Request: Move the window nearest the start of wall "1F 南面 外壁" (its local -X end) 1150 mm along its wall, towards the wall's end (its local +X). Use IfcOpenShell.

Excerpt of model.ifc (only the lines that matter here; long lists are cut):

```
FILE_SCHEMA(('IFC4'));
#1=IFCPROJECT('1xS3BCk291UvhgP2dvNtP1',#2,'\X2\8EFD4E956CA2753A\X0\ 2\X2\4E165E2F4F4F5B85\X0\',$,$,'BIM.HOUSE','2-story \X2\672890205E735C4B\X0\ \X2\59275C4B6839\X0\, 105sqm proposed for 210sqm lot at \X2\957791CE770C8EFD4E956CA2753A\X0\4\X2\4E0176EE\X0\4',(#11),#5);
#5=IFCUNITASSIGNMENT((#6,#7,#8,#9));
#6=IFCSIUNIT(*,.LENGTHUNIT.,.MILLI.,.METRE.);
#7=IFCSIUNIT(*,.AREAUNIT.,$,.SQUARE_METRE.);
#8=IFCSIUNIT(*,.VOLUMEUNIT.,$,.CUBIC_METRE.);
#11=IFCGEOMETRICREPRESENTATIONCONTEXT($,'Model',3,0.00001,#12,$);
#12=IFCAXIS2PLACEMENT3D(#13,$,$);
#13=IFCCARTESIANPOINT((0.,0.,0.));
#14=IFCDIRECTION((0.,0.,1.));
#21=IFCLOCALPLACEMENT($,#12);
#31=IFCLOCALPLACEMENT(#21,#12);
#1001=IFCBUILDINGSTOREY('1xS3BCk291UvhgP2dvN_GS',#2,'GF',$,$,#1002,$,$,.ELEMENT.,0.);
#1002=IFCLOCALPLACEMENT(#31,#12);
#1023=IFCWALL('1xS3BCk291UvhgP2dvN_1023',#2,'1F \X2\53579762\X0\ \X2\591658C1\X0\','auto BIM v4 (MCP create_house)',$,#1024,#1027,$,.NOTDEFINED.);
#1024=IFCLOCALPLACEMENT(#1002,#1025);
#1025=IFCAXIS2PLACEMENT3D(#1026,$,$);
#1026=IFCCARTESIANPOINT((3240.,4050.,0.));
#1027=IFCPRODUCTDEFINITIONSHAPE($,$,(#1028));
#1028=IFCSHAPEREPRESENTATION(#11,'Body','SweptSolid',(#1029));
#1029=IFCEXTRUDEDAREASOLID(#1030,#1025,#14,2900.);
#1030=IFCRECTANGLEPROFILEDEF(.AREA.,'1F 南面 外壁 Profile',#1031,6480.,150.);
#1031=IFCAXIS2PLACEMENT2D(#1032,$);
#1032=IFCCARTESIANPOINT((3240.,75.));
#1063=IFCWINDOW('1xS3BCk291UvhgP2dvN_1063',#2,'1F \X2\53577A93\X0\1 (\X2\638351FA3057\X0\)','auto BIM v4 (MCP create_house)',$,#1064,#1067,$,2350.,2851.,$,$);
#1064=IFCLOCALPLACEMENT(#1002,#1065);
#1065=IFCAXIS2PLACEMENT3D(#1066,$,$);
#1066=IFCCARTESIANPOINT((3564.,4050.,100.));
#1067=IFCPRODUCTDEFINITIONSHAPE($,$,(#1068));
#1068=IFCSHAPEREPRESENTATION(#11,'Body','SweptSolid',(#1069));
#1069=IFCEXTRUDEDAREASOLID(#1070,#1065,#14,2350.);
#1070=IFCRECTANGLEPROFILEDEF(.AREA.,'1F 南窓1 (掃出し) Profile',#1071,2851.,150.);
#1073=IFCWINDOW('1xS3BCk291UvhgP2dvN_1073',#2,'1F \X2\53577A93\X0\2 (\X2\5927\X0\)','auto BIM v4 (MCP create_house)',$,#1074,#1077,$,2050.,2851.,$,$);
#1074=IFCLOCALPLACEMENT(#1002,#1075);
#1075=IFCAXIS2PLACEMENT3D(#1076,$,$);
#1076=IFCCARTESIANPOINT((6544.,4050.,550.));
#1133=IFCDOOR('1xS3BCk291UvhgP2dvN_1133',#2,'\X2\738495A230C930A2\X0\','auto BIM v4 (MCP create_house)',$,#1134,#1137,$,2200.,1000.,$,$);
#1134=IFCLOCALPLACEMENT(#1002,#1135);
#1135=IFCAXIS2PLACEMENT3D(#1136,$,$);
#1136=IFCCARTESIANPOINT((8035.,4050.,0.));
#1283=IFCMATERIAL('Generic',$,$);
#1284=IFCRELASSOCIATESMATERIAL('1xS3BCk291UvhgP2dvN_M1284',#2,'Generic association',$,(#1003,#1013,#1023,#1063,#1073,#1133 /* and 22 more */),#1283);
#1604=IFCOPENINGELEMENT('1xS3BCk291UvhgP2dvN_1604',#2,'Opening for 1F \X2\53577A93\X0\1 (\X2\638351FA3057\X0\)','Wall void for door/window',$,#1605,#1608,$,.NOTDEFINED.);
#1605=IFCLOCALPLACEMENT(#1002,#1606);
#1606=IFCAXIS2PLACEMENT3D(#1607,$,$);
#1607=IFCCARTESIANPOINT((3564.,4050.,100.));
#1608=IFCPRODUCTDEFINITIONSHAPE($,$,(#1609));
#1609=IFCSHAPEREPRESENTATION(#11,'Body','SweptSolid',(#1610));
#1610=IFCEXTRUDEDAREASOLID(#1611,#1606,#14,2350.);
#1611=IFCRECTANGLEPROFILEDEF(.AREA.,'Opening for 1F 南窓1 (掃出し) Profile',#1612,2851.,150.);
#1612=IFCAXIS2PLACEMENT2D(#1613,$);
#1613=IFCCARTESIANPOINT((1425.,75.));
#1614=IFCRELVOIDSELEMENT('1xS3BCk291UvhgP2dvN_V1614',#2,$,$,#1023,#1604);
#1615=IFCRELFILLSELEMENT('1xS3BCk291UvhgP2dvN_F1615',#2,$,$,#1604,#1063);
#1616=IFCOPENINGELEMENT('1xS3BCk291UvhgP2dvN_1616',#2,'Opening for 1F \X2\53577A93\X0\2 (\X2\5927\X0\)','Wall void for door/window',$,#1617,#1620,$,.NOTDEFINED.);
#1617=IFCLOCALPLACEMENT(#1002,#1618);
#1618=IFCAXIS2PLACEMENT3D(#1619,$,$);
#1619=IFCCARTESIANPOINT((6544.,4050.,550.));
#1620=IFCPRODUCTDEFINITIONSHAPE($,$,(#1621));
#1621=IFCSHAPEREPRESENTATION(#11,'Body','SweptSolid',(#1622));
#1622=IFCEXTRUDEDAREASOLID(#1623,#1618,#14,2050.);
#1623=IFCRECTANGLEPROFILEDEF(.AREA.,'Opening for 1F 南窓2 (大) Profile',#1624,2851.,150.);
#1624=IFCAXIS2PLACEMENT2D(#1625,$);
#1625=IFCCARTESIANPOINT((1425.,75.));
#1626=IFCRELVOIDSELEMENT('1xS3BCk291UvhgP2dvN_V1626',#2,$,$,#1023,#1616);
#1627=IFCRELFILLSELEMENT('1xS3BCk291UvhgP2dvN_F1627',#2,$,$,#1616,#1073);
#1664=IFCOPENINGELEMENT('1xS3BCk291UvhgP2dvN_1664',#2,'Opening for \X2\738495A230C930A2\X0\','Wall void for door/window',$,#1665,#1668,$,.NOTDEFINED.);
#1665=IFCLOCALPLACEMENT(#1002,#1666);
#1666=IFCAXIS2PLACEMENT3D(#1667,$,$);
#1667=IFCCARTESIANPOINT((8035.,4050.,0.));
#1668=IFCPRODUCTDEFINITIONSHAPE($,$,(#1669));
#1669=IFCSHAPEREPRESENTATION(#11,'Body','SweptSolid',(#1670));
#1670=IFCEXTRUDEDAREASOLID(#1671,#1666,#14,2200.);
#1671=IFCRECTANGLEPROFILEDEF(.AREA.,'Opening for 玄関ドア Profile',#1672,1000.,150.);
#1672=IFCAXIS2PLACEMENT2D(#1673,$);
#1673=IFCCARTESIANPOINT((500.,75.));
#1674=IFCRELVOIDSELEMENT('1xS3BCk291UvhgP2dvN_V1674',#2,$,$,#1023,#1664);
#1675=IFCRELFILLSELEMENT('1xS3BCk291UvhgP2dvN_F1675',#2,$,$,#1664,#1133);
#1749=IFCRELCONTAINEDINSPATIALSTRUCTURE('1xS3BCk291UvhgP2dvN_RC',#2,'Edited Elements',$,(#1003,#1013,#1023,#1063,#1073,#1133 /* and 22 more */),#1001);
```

```python
import ifcopenshell
import ifcopenshell.api.geometry
import ifcopenshell.util.placement

model = ifcopenshell.open("model.ifc")

window = model.by_guid("1xS3BCk291UvhgP2dvN_1063")
opening = window.FillsVoids[0].RelatingOpeningElement
wall = opening.VoidsElements[0].RelatingBuildingElement

wall_matrix = ifcopenshell.util.placement.get_local_placement(wall.ObjectPlacement)
shift = wall_matrix[:3, 0] * 1150.0
before = ifcopenshell.util.placement.get_local_placement(window.ObjectPlacement)[:3, 3].copy()

# The window is not placed relative to its opening, so move both.
for product in (opening, window):
    matrix = ifcopenshell.util.placement.get_local_placement(product.ObjectPlacement)
    matrix[:3, 3] += shift
    ifcopenshell.api.geometry.edit_object_placement(model, product=product, matrix=matrix, is_si=False)

after = ifcopenshell.util.placement.get_local_placement(window.ObjectPlacement)[:3, 3]
print("window moved by", (after - before).round(3) + 0.0)

model.write("model_rev.ifc")
```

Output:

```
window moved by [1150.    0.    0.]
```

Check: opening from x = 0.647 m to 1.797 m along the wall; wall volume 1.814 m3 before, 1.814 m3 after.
